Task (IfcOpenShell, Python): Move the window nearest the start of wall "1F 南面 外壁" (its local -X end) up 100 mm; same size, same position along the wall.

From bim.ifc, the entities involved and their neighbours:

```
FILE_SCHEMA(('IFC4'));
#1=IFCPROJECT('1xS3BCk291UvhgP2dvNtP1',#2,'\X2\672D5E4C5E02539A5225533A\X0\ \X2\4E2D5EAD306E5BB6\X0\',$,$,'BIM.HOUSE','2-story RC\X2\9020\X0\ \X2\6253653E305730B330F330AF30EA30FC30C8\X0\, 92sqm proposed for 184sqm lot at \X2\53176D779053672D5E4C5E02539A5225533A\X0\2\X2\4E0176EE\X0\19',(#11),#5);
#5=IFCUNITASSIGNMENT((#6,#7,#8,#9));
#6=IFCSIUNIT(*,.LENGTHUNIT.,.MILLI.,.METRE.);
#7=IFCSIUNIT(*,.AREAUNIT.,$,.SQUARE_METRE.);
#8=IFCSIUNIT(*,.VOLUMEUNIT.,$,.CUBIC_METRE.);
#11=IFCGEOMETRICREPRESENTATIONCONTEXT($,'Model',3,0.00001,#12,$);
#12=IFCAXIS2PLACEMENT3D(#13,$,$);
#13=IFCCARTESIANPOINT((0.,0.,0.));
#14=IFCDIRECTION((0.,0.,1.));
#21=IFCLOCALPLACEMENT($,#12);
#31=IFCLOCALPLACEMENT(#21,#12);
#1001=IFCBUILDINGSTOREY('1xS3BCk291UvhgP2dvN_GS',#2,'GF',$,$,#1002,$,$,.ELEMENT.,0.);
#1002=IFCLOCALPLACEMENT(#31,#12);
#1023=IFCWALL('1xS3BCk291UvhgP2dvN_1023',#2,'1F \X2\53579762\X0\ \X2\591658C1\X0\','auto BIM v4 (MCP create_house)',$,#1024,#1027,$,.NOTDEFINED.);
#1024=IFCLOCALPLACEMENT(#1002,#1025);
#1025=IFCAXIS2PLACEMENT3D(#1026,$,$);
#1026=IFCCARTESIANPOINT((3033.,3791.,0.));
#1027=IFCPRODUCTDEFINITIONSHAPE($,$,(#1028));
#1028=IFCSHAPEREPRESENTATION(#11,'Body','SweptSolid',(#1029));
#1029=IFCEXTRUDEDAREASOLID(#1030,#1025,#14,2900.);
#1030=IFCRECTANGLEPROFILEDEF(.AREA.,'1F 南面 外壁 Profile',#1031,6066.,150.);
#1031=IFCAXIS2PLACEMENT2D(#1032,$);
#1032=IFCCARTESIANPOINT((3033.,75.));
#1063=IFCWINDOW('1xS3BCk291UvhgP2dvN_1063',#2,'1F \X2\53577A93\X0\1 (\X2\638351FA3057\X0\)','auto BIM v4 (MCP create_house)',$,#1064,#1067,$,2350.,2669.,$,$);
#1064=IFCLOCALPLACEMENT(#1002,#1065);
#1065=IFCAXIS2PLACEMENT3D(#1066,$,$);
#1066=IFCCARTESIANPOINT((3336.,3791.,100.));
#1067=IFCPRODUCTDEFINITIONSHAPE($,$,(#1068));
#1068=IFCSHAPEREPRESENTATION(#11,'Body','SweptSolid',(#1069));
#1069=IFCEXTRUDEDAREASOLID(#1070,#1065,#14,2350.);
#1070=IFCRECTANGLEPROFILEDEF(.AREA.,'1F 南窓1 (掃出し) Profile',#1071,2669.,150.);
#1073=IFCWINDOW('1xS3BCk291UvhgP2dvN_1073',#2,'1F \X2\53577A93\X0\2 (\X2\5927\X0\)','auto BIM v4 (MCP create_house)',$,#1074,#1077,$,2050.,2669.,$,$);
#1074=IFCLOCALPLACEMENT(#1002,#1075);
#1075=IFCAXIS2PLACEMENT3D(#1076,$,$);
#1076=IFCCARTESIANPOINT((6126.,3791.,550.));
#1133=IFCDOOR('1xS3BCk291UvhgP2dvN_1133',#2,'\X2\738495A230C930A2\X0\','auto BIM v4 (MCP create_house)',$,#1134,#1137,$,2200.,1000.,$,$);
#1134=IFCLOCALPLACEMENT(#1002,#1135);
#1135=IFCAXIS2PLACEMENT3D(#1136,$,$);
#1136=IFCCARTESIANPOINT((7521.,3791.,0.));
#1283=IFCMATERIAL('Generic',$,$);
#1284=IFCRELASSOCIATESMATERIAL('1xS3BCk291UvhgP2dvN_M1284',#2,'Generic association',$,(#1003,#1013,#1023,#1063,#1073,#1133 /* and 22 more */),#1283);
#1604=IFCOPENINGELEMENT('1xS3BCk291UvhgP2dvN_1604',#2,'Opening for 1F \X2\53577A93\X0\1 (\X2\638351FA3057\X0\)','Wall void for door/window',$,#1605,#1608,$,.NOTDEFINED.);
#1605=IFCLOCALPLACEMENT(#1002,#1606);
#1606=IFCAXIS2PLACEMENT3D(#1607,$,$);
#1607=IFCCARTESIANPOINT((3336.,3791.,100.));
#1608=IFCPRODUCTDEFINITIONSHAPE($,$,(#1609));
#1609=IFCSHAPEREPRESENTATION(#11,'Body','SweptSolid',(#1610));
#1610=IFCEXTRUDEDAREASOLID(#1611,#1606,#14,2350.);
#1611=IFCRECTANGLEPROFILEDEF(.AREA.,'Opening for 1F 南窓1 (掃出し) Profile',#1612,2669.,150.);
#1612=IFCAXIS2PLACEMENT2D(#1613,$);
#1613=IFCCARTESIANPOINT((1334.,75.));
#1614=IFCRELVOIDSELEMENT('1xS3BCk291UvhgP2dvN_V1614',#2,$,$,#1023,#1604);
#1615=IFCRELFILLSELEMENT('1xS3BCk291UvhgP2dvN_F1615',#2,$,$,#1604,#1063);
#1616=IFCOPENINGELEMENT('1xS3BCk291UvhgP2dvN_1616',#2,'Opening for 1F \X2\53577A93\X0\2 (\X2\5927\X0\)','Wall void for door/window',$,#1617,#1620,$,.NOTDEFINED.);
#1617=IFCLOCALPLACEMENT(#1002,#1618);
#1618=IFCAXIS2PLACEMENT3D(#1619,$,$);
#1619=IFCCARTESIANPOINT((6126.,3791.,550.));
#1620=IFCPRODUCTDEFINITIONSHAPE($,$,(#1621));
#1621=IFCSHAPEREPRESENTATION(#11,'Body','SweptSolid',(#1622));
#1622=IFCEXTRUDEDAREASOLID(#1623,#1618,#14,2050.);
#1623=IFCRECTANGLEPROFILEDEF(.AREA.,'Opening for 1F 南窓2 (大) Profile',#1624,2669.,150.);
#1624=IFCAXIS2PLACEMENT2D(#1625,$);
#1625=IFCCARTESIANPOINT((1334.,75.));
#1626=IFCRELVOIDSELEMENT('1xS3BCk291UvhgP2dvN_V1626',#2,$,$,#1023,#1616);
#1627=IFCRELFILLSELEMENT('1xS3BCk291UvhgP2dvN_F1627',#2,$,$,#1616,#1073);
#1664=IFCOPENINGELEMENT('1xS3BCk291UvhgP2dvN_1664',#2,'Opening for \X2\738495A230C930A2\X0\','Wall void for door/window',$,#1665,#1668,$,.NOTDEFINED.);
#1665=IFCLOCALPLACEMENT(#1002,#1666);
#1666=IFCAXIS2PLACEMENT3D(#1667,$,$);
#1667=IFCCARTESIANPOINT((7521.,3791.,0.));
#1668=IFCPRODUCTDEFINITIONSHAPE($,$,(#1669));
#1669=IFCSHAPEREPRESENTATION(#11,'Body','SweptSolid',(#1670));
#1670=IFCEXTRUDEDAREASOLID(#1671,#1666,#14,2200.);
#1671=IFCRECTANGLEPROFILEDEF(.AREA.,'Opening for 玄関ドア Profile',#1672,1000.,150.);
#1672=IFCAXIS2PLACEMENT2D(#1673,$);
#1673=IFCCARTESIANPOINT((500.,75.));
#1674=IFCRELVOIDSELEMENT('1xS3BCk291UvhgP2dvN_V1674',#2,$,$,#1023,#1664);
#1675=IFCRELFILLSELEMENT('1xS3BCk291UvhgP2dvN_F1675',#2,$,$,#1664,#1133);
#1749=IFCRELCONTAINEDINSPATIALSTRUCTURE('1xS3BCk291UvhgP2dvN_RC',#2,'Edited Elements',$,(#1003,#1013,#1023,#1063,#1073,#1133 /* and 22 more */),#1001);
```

```python
import numpy as np
import ifcopenshell
import ifcopenshell.api.geometry
import ifcopenshell.util.placement
import ifcopenshell.util.unit

model = ifcopenshell.open("bim.ifc")
unit_scale = ifcopenshell.util.unit.calculate_unit_scale(model)

window = model.by_guid("1xS3BCk291UvhgP2dvN_1063")
opening = window.FillsVoids[0].RelatingOpeningElement
dz = 100.0

shift = np.array([0.0, 0.0, dz])
# The window is not placed relative to its opening, so move both.
for product in (opening, window):
    matrix = ifcopenshell.util.placement.get_local_placement(product.ObjectPlacement)
    matrix[:3, 3] += shift
    ifcopenshell.api.geometry.edit_object_placement(model, product=product, matrix=matrix, is_si=False)

print(f"moved by {dz * unit_scale:+.3f} m")

model.write("bim_updated.ifc")
```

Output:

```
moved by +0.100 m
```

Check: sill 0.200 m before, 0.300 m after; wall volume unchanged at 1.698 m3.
